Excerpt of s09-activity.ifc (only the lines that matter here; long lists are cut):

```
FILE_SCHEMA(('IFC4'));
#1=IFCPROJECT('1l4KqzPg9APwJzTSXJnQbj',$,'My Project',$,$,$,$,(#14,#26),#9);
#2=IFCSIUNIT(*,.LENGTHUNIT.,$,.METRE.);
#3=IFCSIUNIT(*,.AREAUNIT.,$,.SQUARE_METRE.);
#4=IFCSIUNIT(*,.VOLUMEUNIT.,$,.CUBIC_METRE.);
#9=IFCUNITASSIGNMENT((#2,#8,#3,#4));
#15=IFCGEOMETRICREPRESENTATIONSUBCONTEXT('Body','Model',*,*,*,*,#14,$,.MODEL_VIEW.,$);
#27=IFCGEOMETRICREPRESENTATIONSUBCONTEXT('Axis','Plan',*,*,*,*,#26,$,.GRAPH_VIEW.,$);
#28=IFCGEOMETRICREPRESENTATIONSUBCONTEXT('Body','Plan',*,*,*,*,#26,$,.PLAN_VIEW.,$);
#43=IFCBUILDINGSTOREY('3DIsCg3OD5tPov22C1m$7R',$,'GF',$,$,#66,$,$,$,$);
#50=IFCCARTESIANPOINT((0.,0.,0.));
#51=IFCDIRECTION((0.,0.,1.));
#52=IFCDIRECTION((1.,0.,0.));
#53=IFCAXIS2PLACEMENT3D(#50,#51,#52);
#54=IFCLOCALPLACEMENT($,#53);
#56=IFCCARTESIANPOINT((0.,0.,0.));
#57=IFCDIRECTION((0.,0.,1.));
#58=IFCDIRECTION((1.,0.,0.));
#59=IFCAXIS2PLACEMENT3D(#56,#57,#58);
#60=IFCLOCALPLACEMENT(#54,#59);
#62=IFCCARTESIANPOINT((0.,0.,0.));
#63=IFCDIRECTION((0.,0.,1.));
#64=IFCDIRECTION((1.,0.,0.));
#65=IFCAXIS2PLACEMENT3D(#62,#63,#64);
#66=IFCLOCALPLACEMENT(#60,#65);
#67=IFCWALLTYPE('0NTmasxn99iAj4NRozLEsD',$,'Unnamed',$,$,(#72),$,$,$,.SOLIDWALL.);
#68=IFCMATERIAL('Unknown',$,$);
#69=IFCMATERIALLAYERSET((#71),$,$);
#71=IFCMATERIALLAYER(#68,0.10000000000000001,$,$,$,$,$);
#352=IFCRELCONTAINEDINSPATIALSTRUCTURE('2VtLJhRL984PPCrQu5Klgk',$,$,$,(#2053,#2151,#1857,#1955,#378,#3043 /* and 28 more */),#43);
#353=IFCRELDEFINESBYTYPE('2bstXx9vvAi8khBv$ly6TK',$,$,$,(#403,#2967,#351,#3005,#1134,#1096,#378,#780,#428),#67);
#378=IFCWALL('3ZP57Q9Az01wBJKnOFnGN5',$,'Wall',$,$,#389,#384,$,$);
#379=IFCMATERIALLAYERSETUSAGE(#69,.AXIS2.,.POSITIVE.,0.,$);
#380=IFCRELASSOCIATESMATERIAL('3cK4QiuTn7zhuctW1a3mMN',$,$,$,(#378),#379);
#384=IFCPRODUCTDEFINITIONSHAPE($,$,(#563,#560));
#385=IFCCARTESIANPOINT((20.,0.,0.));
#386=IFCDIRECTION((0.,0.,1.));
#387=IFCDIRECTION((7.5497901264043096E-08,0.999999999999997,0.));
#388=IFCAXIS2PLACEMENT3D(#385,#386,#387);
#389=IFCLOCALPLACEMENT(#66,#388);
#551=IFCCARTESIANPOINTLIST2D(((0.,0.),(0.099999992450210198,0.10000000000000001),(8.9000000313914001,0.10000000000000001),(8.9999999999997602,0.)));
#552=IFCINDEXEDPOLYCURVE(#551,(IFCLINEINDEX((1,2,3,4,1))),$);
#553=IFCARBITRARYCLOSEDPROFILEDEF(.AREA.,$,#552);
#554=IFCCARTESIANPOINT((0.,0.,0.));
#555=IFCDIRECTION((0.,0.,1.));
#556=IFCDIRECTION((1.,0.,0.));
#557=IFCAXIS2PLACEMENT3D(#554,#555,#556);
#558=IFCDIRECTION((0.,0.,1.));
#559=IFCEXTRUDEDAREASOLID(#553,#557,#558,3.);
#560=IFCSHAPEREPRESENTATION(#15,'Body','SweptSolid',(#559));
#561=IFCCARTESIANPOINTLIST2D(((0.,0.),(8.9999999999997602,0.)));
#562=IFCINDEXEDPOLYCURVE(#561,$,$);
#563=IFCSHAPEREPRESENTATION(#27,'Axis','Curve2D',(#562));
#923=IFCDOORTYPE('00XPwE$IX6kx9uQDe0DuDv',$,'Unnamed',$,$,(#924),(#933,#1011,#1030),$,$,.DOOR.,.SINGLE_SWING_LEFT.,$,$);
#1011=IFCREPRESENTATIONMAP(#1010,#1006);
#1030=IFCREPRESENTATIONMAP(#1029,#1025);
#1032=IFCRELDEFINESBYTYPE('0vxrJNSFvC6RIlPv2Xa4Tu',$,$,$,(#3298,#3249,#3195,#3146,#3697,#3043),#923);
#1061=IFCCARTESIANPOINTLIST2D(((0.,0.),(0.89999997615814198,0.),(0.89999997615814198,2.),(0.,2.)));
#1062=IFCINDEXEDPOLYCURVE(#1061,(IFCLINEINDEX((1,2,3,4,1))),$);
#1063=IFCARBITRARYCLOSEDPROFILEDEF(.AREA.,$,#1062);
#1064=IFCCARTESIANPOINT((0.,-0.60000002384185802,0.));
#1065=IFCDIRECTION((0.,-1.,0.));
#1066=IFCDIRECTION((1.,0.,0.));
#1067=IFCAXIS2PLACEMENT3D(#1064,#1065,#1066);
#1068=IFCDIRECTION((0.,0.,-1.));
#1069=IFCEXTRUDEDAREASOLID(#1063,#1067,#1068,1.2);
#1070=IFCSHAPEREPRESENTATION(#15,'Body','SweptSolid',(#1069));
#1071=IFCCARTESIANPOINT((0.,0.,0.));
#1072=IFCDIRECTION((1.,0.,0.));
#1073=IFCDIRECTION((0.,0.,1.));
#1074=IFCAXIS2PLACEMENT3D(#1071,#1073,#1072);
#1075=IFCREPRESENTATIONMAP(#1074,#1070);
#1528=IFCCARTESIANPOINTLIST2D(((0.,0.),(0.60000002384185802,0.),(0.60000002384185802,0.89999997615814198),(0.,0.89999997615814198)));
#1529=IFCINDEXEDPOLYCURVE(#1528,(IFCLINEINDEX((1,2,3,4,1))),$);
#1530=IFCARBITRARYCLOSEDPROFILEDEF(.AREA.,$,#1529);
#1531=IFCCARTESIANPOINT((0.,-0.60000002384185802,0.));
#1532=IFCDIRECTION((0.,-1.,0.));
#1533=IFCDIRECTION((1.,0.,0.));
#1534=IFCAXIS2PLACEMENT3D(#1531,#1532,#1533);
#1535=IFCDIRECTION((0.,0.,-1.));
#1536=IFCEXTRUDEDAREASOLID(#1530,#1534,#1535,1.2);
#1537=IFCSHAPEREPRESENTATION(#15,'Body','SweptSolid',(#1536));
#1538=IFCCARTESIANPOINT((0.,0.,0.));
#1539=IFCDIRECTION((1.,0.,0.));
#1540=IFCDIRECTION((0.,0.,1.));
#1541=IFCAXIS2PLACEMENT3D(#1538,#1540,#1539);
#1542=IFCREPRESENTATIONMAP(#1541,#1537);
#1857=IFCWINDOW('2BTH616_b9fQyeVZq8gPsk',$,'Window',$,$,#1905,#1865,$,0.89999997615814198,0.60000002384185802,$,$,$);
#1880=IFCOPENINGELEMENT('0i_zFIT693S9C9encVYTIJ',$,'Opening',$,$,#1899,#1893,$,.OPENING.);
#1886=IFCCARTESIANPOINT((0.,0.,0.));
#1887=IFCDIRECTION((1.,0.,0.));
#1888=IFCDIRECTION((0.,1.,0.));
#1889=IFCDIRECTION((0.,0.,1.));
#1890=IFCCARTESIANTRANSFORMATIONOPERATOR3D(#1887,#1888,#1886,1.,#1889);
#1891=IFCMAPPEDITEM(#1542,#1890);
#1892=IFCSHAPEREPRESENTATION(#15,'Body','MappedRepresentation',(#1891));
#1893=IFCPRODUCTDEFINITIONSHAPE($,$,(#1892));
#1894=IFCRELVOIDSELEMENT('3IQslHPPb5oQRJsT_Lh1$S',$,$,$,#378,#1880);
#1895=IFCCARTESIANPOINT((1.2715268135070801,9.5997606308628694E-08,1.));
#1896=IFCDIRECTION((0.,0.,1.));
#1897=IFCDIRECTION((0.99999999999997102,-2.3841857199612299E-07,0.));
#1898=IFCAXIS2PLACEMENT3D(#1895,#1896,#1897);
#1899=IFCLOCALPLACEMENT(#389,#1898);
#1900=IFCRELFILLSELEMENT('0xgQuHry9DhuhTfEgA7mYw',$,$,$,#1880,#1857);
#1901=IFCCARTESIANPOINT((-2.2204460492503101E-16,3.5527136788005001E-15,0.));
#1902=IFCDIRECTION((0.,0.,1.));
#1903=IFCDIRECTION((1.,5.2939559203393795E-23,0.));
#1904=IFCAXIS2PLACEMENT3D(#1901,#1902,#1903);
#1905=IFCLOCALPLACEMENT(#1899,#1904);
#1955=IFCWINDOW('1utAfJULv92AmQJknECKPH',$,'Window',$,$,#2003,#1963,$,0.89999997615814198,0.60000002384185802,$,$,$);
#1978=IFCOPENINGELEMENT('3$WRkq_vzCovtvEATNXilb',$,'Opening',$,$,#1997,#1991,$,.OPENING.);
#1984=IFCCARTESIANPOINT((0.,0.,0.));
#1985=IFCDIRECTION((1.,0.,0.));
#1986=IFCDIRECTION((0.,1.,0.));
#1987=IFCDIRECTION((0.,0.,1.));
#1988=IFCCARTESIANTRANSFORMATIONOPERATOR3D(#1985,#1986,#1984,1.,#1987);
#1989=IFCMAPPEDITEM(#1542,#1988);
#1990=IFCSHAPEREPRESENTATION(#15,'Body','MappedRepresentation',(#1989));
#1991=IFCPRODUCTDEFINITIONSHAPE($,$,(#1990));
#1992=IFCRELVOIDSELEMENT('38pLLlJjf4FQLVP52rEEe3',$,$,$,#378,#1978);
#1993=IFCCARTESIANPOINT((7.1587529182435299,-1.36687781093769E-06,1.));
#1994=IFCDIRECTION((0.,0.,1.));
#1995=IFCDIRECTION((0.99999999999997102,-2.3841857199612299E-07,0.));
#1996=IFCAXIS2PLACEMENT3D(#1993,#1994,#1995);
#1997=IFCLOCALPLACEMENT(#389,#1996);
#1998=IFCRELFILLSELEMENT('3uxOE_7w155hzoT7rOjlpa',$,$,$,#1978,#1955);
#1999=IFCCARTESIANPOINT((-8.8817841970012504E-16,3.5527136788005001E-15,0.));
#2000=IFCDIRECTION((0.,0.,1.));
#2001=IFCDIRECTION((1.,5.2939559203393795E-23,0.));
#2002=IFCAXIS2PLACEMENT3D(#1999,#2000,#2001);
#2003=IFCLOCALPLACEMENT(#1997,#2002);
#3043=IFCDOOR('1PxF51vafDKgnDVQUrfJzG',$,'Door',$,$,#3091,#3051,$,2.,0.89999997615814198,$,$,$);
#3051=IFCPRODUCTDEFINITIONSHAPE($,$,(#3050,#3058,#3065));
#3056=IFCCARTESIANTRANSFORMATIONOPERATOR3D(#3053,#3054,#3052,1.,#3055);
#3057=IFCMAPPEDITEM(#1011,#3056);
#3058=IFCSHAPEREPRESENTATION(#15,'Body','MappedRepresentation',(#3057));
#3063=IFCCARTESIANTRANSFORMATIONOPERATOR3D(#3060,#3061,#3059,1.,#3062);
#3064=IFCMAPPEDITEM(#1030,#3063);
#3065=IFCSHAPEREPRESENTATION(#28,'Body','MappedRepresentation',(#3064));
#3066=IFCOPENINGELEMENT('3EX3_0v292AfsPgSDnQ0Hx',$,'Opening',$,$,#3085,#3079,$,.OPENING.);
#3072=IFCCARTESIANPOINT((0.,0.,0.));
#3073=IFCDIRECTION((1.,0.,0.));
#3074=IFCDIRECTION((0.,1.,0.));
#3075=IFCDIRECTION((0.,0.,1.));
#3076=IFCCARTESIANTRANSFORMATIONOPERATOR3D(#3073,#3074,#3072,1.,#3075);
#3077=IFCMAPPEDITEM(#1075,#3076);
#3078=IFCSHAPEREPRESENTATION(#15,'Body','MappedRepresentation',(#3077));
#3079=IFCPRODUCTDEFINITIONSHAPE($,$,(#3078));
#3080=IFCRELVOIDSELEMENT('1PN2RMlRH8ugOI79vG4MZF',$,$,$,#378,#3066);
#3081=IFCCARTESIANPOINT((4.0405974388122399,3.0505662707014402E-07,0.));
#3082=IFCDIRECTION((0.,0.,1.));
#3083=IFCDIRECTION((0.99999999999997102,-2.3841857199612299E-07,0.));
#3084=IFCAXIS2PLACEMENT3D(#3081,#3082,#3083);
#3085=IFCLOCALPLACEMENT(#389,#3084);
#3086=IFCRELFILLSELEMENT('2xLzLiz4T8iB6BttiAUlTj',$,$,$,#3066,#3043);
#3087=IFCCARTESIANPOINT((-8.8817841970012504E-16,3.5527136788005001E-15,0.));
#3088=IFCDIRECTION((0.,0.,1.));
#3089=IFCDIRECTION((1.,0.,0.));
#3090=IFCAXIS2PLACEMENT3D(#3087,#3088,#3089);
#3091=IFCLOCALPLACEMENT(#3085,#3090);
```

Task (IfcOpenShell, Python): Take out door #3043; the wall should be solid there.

```python
import ifcopenshell
import ifcopenshell.api.feature
import ifcopenshell.api.root
import ifcopenshell.geom
import ifcopenshell.util.shape

model = ifcopenshell.open("s09-activity.ifc")
settings = ifcopenshell.geom.settings()


def volume(element):
    """Net volume in cubic metres, openings subtracted."""
    shape = ifcopenshell.geom.create_shape(settings, element)
    return ifcopenshell.util.shape.get_volume(shape.geometry)


door = model.by_guid("1PxF51vafDKgnDVQUrfJzG")
opening = door.FillsVoids[0].RelatingOpeningElement
wall = opening.VoidsElements[0].RelatingBuildingElement
before = volume(wall)

ifcopenshell.api.root.remove_product(model, product=door)
ifcopenshell.api.feature.remove_feature(model, feature=opening)

after = volume(wall)

print(f"wall volume {before:.3f} -> {after:.3f} m3")

model.write("s09-activity_updated.ifc")
```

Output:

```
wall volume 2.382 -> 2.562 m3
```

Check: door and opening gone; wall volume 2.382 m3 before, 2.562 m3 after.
